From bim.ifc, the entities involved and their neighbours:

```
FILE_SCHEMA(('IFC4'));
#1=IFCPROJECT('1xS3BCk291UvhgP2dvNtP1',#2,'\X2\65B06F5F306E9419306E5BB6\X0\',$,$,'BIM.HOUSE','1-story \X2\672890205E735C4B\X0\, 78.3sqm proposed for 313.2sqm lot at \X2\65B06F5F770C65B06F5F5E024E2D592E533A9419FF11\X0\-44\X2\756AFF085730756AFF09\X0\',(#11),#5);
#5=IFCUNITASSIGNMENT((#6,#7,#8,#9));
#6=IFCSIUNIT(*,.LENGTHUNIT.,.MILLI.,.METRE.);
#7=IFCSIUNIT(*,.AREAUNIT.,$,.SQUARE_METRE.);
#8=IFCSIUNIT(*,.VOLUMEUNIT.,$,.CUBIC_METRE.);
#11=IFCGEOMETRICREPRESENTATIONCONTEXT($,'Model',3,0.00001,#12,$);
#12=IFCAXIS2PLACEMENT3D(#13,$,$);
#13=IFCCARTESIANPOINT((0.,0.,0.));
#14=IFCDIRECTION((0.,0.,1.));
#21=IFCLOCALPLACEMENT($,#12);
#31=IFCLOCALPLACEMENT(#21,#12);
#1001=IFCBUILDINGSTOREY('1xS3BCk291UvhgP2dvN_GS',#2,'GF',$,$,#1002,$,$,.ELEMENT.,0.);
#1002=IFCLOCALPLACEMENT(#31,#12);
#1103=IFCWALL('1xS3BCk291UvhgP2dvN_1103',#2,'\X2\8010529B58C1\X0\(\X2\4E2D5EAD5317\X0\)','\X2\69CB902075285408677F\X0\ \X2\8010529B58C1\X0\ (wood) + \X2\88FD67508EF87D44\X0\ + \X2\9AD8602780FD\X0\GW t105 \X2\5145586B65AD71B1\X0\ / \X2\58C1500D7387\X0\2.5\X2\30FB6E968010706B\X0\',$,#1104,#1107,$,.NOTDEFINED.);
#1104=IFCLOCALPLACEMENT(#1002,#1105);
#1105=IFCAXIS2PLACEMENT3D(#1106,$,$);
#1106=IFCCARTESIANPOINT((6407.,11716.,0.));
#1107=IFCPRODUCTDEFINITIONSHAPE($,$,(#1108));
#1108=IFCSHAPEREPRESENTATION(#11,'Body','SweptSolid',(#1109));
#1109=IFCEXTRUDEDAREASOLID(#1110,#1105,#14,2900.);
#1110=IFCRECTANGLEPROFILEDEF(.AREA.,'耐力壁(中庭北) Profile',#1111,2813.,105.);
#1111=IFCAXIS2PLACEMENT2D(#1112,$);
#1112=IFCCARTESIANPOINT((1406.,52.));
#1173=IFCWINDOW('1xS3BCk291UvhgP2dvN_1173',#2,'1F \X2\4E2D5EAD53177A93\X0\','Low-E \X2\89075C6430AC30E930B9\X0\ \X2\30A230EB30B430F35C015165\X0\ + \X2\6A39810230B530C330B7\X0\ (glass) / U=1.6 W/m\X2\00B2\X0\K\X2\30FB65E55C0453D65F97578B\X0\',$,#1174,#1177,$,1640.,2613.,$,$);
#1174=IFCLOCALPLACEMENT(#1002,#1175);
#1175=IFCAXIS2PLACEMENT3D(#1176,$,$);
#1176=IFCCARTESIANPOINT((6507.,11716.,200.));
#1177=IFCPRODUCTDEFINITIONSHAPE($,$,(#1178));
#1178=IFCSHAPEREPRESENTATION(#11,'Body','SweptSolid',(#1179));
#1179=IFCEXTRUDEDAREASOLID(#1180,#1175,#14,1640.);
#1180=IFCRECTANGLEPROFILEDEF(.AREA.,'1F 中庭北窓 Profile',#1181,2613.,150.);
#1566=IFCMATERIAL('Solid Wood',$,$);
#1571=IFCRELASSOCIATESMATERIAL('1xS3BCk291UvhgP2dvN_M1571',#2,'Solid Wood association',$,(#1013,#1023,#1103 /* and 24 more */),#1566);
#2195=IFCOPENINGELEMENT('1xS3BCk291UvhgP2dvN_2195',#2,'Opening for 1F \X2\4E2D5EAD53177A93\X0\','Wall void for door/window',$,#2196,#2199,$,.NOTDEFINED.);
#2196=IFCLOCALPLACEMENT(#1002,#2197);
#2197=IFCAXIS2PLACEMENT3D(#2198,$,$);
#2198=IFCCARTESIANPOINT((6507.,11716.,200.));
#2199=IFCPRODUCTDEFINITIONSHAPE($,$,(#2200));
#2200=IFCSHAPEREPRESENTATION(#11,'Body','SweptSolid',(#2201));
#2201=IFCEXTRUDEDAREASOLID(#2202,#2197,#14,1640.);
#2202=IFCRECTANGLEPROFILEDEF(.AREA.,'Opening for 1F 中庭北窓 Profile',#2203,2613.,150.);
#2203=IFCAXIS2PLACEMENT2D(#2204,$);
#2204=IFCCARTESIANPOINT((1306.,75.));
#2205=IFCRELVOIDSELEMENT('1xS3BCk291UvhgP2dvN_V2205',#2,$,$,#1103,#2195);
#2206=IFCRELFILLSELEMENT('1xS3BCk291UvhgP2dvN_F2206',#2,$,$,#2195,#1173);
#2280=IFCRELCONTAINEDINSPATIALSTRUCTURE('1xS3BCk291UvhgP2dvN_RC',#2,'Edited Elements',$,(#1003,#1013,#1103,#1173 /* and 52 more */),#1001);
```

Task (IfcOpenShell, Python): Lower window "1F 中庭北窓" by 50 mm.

```python
import numpy as np
import ifcopenshell
import ifcopenshell.api.geometry
import ifcopenshell.util.placement
import ifcopenshell.util.unit

model = ifcopenshell.open("bim.ifc")
unit_scale = ifcopenshell.util.unit.calculate_unit_scale(model)

window = model.by_id(1173)
opening = window.FillsVoids[0].RelatingOpeningElement
dz = -0.05 / unit_scale

shift = np.array([0.0, 0.0, dz])
# The window is not placed relative to its opening, so move both.
for product in (opening, window):
    matrix = ifcopenshell.util.placement.get_local_placement(product.ObjectPlacement)
    matrix[:3, 3] += shift
    ifcopenshell.api.geometry.edit_object_placement(model, product=product, matrix=matrix, is_si=False)

print(f"moved by {dz * unit_scale:+.3f} m")

model.write("bim_rev.ifc")
```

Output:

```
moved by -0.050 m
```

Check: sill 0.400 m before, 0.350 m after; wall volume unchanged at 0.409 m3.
